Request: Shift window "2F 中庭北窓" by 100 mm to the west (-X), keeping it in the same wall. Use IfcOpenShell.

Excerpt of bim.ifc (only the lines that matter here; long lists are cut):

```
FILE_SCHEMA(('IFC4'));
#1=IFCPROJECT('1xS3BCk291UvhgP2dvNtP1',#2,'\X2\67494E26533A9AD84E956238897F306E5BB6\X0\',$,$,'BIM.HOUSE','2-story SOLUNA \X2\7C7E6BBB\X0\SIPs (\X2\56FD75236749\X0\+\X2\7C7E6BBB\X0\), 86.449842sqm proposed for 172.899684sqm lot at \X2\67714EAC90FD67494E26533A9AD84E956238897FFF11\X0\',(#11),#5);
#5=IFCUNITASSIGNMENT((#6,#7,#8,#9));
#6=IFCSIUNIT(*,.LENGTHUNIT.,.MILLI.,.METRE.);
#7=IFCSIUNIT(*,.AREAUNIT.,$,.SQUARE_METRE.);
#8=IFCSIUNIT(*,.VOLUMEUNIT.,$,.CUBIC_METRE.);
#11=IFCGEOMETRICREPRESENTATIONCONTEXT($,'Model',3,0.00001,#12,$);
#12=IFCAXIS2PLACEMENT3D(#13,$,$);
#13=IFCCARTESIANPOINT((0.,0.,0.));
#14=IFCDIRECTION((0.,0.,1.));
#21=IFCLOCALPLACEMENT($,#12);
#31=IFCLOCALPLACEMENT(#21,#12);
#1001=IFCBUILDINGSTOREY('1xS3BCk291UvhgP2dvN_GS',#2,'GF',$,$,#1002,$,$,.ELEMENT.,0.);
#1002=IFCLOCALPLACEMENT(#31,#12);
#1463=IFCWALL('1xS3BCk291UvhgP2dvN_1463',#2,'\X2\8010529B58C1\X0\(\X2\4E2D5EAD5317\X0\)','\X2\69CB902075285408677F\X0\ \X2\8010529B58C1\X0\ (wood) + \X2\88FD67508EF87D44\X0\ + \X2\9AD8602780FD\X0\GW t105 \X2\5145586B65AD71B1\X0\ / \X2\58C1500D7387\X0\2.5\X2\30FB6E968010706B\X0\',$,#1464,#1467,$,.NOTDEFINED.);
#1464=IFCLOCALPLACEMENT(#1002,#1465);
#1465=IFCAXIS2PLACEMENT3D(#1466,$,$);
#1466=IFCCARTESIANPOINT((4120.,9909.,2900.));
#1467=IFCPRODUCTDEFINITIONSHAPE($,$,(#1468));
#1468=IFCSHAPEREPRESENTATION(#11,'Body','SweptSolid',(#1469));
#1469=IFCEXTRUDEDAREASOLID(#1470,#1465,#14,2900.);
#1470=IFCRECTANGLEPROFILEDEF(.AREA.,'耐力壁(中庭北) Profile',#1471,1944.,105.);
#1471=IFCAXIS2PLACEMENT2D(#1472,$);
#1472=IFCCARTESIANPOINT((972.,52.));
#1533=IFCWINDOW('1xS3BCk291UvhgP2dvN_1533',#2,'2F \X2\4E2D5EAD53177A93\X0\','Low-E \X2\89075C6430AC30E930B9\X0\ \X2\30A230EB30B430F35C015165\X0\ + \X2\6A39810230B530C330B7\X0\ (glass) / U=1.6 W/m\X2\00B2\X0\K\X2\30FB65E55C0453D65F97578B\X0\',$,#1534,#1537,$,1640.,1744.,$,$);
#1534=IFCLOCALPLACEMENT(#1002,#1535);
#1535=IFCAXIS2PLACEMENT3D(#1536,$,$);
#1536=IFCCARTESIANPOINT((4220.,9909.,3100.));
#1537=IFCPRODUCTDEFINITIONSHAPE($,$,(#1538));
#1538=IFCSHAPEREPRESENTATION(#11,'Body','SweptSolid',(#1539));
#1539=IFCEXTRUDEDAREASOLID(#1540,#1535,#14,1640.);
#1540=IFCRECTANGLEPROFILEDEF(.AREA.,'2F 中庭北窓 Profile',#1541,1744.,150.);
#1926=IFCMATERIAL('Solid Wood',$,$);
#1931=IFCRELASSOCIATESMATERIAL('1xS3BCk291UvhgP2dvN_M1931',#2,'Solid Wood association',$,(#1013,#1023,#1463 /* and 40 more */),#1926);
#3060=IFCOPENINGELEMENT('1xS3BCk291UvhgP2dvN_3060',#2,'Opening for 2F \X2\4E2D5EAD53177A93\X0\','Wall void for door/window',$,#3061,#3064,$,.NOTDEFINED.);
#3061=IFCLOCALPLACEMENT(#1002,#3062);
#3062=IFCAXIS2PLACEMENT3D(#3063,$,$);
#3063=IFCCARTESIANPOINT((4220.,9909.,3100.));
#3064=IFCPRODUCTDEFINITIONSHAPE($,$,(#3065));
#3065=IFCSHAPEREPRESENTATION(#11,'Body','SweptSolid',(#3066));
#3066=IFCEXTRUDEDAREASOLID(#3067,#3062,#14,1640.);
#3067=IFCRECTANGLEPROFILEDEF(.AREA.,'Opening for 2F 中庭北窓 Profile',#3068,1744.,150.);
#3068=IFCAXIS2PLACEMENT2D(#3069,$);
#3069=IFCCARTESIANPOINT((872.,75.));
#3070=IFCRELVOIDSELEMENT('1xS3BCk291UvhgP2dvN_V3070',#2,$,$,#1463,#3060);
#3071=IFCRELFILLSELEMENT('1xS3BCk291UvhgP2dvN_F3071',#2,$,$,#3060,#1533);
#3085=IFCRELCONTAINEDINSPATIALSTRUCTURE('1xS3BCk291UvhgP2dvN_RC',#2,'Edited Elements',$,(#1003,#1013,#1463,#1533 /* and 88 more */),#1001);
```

```python
import ifcopenshell
import ifcopenshell.api.geometry
import ifcopenshell.util.placement
import ifcopenshell.util.unit

model = ifcopenshell.open("bim.ifc")
unit_scale = ifcopenshell.util.unit.calculate_unit_scale(model)

window = model.by_guid("1xS3BCk291UvhgP2dvN_1533")
opening = window.FillsVoids[0].RelatingOpeningElement
wall = opening.VoidsElements[0].RelatingBuildingElement

wall_matrix = ifcopenshell.util.placement.get_local_placement(wall.ObjectPlacement)
shift = wall_matrix[:3, 0] * -0.1 / unit_scale
before = ifcopenshell.util.placement.get_local_placement(window.ObjectPlacement)[:3, 3].copy()

# The window is not placed relative to its opening, so move both.
for product in (opening, window):
    matrix = ifcopenshell.util.placement.get_local_placement(product.ObjectPlacement)
    matrix[:3, 3] += shift
    ifcopenshell.api.geometry.edit_object_placement(model, product=product, matrix=matrix, is_si=False)

after = ifcopenshell.util.placement.get_local_placement(window.ObjectPlacement)[:3, 3]
print("window moved by", (after - before).round(3) + 0.0)

model.write("bim_edited.ifc")
```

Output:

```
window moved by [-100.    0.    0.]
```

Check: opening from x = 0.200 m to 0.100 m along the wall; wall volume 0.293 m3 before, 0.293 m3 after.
